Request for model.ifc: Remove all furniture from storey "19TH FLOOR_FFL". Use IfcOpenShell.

First a look at what the model holds.

```python
import ifcopenshell
import ifcopenshell.util.element

model = ifcopenshell.open("model.ifc")
print(model.schema)
storey = next(s for s in model.by_type("IfcBuildingStorey") if s.Name == "19TH FLOOR_FFL")
furniture = [e for e in ifcopenshell.util.element.get_decomposition(storey) if e.is_a("IfcFurnishingElement")]
seen = {}
for e in furniture:
    element_type = ifcopenshell.util.element.get_type(e)
    name = element_type.Name if element_type not in (None, e) else None
    seen[name] = seen.get(name, 0) + 1
for name, count in sorted(seen.items(), key=str):
    print(count, "x", name)
```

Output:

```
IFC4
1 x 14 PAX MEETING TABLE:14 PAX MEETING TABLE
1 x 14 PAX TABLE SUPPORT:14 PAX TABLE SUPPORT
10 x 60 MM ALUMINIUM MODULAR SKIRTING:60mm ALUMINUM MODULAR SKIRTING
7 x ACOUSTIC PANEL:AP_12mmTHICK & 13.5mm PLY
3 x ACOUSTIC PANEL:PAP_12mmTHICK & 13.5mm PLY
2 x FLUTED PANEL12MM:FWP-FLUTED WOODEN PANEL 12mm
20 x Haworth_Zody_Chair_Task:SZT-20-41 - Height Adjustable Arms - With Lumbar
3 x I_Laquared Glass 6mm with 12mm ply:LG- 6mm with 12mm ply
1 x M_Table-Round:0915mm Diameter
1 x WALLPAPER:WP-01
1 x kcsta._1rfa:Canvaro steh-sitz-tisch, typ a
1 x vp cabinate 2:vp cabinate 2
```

```python
import ifcopenshell
import ifcopenshell.api.root
import ifcopenshell.util.element

model = ifcopenshell.open("model.ifc")

storey = next(s for s in model.by_type("IfcBuildingStorey") if s.Name == "19TH FLOOR_FFL")
furniture = [e for e in ifcopenshell.util.element.get_decomposition(storey) if e.is_a("IfcFurnishingElement")]

for e in furniture:
    ifcopenshell.api.root.remove_product(model, product=e)
print(len(furniture), "removed")

model.write("model_updated.ifc")
```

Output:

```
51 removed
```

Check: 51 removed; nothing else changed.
